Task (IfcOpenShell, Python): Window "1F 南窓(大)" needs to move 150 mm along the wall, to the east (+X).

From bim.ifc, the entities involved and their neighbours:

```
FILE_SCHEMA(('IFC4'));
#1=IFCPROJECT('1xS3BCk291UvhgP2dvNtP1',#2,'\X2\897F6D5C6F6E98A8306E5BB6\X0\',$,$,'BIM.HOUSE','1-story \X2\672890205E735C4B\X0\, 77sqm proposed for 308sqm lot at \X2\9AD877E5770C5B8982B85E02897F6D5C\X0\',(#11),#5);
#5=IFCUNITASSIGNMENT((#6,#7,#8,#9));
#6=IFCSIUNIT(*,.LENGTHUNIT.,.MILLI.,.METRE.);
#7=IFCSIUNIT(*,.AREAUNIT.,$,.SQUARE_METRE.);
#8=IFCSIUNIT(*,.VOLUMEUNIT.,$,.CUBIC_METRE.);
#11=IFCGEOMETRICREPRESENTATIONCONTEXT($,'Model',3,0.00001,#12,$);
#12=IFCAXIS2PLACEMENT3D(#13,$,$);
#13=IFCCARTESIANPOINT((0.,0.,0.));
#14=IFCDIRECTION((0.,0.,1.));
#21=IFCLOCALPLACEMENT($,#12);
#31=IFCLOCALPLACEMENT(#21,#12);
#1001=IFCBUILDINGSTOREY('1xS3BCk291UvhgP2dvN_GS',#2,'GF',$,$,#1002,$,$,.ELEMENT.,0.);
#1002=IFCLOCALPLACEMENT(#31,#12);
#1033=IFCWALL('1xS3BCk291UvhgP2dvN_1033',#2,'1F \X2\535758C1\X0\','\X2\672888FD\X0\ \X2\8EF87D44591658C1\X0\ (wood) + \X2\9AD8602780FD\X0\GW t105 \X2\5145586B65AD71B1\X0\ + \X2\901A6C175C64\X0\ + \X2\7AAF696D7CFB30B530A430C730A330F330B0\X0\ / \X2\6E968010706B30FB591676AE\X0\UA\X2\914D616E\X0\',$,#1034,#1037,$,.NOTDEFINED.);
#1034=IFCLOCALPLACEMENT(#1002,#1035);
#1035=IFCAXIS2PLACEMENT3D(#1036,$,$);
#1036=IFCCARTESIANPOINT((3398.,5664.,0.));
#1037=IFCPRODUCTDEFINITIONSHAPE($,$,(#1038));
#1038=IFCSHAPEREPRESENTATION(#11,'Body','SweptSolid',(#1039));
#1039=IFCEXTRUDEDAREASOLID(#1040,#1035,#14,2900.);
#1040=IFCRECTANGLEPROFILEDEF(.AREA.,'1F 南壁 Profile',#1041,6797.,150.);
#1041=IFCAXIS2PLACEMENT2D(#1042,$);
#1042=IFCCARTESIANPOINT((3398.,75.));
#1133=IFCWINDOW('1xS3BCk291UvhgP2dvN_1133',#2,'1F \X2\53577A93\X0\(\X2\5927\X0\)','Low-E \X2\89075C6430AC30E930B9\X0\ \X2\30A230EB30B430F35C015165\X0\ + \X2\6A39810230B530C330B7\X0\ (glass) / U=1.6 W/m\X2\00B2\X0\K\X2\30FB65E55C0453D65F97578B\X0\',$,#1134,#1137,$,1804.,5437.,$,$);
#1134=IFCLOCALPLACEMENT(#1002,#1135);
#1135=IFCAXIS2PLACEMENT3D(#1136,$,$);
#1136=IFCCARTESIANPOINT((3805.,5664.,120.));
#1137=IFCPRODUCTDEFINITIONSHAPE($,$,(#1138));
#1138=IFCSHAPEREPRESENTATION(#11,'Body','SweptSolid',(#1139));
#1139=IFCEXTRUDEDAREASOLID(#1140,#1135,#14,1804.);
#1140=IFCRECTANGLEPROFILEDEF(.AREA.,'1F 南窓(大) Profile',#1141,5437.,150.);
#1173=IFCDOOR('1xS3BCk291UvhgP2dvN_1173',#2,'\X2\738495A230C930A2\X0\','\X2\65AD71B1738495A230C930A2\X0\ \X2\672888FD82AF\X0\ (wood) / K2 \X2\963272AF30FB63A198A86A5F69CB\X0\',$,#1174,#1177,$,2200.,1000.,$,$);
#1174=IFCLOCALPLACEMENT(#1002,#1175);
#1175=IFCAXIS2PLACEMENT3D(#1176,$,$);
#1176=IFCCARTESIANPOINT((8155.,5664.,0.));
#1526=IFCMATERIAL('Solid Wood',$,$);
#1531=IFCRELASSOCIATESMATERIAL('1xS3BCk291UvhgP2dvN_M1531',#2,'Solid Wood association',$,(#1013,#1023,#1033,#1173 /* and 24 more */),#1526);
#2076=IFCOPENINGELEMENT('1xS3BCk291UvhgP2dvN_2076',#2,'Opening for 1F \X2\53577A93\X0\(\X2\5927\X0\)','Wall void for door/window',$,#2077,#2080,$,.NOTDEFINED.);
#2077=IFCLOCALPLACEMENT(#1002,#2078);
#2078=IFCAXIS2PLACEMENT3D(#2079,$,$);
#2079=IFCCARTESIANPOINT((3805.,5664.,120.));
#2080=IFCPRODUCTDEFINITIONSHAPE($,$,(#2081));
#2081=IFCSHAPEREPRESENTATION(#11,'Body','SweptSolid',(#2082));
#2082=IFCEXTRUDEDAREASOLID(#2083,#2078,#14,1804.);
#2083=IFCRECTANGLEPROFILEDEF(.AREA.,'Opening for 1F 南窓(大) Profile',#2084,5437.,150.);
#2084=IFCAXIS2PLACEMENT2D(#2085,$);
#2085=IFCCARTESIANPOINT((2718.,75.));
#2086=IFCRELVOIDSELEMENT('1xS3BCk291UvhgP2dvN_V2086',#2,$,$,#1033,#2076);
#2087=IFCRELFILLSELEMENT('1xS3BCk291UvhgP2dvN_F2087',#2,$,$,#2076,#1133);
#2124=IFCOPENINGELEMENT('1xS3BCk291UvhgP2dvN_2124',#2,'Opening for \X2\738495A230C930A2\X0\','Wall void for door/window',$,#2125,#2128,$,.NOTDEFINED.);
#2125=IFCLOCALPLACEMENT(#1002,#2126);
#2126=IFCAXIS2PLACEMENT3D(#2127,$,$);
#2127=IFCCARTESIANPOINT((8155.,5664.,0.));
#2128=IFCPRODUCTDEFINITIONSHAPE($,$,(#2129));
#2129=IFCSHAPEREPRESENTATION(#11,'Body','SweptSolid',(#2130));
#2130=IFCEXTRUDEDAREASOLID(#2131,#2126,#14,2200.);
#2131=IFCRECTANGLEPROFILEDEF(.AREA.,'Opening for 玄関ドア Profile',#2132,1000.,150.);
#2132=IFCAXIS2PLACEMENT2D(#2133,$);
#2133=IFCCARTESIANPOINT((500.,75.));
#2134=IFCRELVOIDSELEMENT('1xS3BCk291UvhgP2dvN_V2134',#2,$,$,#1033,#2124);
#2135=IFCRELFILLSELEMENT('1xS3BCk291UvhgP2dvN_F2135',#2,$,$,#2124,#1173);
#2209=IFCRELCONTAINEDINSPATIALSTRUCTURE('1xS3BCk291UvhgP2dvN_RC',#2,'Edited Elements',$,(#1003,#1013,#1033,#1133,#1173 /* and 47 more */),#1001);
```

```python
import ifcopenshell
import ifcopenshell.api.geometry
import ifcopenshell.util.placement
import ifcopenshell.util.unit

model = ifcopenshell.open("bim.ifc")
unit_scale = ifcopenshell.util.unit.calculate_unit_scale(model)

window = model.by_guid("1xS3BCk291UvhgP2dvN_1133")
opening = window.FillsVoids[0].RelatingOpeningElement
wall = opening.VoidsElements[0].RelatingBuildingElement

wall_matrix = ifcopenshell.util.placement.get_local_placement(wall.ObjectPlacement)
shift = wall_matrix[:3, 0] * 0.15 / unit_scale
before = ifcopenshell.util.placement.get_local_placement(window.ObjectPlacement)[:3, 3].copy()

# The window is not placed relative to its opening, so move both.
for product in (opening, window):
    matrix = ifcopenshell.util.placement.get_local_placement(product.ObjectPlacement)
    matrix[:3, 3] += shift
    ifcopenshell.api.geometry.edit_object_placement(model, product=product, matrix=matrix, is_si=False)

after = ifcopenshell.util.placement.get_local_placement(window.ObjectPlacement)[:3, 3]
print("window moved by", (after - before).round(3) + 0.0)

model.write("bim_updated.ifc")
```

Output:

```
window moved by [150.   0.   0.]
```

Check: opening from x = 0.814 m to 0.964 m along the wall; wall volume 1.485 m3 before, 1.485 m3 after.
